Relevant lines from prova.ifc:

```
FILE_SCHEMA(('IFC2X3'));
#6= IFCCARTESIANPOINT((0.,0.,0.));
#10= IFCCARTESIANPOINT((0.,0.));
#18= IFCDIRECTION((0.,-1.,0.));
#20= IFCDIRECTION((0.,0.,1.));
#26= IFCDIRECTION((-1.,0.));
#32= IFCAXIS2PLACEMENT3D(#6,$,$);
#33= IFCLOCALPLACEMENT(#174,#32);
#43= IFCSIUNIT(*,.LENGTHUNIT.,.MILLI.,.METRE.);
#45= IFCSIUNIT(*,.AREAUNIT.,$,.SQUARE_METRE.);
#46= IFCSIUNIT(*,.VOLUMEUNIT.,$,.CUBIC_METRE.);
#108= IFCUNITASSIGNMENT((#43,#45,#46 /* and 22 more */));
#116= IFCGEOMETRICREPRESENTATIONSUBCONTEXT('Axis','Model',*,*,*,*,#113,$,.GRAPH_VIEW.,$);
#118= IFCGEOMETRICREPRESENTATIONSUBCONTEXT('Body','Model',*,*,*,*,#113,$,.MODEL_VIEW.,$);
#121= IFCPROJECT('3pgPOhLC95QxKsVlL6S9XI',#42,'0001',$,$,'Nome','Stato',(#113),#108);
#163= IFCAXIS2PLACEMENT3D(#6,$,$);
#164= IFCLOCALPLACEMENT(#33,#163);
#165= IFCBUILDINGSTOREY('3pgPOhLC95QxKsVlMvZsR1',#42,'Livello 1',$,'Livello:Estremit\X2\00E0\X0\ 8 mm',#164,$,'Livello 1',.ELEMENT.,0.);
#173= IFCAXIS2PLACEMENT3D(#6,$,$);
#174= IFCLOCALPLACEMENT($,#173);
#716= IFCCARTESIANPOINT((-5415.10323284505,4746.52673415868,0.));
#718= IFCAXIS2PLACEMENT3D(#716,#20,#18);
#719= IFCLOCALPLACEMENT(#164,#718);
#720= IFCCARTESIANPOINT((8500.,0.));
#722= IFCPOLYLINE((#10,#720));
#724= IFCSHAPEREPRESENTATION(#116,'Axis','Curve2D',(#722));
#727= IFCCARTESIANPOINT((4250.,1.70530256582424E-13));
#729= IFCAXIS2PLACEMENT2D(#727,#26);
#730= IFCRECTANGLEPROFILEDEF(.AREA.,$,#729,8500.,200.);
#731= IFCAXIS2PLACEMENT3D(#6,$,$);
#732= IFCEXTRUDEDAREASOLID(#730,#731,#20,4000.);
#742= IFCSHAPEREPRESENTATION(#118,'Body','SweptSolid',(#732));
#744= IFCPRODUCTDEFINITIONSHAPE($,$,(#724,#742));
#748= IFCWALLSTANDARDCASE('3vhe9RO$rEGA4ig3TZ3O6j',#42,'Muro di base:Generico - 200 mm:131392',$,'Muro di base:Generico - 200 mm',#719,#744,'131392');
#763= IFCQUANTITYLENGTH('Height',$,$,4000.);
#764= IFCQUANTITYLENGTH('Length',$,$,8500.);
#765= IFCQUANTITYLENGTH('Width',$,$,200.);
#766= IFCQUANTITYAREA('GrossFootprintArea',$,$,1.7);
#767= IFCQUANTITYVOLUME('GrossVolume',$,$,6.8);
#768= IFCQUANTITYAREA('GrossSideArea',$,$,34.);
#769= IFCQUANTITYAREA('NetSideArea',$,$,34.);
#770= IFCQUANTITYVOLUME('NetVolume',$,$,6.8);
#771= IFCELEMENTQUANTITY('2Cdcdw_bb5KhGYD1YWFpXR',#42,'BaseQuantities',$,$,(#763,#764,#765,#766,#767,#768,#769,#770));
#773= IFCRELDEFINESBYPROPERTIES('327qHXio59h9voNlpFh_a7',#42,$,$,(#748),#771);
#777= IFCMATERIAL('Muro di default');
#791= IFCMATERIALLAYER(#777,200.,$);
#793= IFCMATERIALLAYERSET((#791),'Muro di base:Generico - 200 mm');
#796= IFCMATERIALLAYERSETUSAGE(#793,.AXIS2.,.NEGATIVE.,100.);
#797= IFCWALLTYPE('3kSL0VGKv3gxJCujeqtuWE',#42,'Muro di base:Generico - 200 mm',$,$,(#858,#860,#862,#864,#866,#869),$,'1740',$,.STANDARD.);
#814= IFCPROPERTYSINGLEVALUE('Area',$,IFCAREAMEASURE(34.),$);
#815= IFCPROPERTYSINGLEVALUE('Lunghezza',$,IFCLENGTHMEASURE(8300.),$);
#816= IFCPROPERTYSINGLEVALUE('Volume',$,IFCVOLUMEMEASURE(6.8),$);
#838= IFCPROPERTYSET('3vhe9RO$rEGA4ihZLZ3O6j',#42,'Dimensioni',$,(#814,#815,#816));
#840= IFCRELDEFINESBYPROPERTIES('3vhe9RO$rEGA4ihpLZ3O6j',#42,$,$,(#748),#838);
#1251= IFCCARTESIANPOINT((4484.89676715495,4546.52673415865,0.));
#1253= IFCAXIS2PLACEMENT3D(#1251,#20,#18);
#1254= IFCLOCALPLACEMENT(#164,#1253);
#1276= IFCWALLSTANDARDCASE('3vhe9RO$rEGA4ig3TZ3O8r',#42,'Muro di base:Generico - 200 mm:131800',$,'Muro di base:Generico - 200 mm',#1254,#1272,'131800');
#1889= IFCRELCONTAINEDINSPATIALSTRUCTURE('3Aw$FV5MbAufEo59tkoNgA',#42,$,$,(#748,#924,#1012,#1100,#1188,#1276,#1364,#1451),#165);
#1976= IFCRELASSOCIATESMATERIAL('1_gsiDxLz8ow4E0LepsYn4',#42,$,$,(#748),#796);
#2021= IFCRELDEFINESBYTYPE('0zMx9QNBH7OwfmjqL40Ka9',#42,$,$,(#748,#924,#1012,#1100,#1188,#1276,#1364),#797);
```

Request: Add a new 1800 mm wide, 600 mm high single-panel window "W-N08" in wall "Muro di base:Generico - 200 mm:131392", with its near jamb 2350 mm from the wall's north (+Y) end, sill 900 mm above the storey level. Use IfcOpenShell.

```python
import numpy as np
import ifcopenshell
import ifcopenshell.api.feature
import ifcopenshell.api.geometry
import ifcopenshell.api.pset
import ifcopenshell.api.root
import ifcopenshell.api.spatial
import ifcopenshell.api.type
import ifcopenshell.geom
import ifcopenshell.util.element
import ifcopenshell.util.placement
import ifcopenshell.util.representation
import ifcopenshell.util.shape
import ifcopenshell.util.unit

model = ifcopenshell.open("prova.ifc")
unit_scale = ifcopenshell.util.unit.calculate_unit_scale(model)
area_scale = ifcopenshell.util.unit.calculate_unit_scale(model, "AREAUNIT")
volume_scale = ifcopenshell.util.unit.calculate_unit_scale(model, "VOLUMEUNIT")
settings = ifcopenshell.geom.settings()


def volume(element):
    """Net volume in cubic metres, openings subtracted."""
    shape = ifcopenshell.geom.create_shape(settings, element)
    return ifcopenshell.util.shape.get_volume(shape.geometry)


wall = model.by_guid("3vhe9RO$rEGA4ig3TZ3O6j")
storey = ifcopenshell.util.element.get_container(wall, ifc_class="IfcBuildingStorey")
context = ifcopenshell.util.representation.get_context(model, "Model", "Body", "MODEL_VIEW")
before = volume(wall)

width, height, from_end, sill = 1.8, 0.6, 2.35, 0.9  # metres

# The wall runs along its own X axis, and the end named is its -X end.
wall_shape = ifcopenshell.geom.create_shape(settings, wall)
x, y, z = ifcopenshell.util.shape.get_vertices(wall_shape.geometry).T
start = x.min() + from_end
face, thickness = float(y.min()), float(y.max() - y.min())
wall_matrix = ifcopenshell.util.placement.get_local_placement(wall.ObjectPlacement)
level = ifcopenshell.util.placement.get_local_placement(storey.ObjectPlacement)[2, 3]


def in_wall(x, y):
    """Placement at x, y metres in the wall's axes, at sill height."""
    matrix = wall_matrix.copy()
    matrix[:, 3] = wall_matrix @ np.array([x / unit_scale, y / unit_scale, 0.0, 1.0])
    matrix[2, 3] = level + sill / unit_scale
    return matrix


# Opening: a box that overshoots both wall faces by 50 mm.
opening = ifcopenshell.api.root.create_entity(model, ifc_class="IfcOpeningElement")
box = ifcopenshell.api.geometry.add_wall_representation(
    model, context=context, length=width, height=height, thickness=thickness + 0.1
)
ifcopenshell.api.geometry.assign_representation(model, product=opening, representation=box)
ifcopenshell.api.geometry.edit_object_placement(model, product=opening, matrix=in_wall(start, face - 0.05), is_si=False)
ifcopenshell.api.feature.add_feature(model, feature=opening, element=wall)

window = ifcopenshell.api.root.create_entity(model, ifc_class="IfcWindow", name="W-N08")
window.OverallWidth, window.OverallHeight = width / unit_scale, height / unit_scale
body = ifcopenshell.api.geometry.add_window_representation(
    model,
    context=context,
    overall_width=window.OverallWidth,
    overall_height=window.OverallHeight,
    partition_type="SINGLE_PANEL",
)
ifcopenshell.api.geometry.assign_representation(model, product=window, representation=body)
ifcopenshell.api.spatial.assign_container(model, products=[window], relating_structure=storey)
fills = ifcopenshell.api.feature.add_filling(model, opening=opening, element=window)
fills.OwnerHistory = window.OwnerHistory  # required in IFC2X3

# IFC2X3 keeps the operation on the window style.
style = ifcopenshell.api.root.create_entity(model, ifc_class="IfcWindowStyle", name="W-N08")
style.OperationType, style.ConstructionType = "SINGLE_PANEL", "NOTDEFINED"
style.ParameterTakesPrecedence = style.Sizeable = False
ifcopenshell.api.type.assign_type(model, related_objects=[window], relating_type=style)

# Centre the window in the wall's thickness.
ifcopenshell.api.geometry.edit_object_placement(model, product=window, matrix=in_wall(start, face), is_si=False)
window_shape = ifcopenshell.geom.create_shape(settings, window)
depth = ifcopenshell.util.shape.get_vertices(window_shape.geometry)[:, 1]
offset = face + thickness / 2 - (depth.min() + depth.max()) / 2
ifcopenshell.api.geometry.edit_object_placement(model, product=window, matrix=in_wall(start, offset), is_si=False)

after = volume(wall)

# Update the wall's stored quantities.
qto = model.by_id(ifcopenshell.util.element.get_pset(wall, "BaseQuantities", should_inherit=False)["id"])
ifcopenshell.api.pset.edit_qto(model, qto=qto, properties={
    "NetSideArea": after / thickness / area_scale,
    "NetVolume": after / volume_scale,
})
pset = model.by_id(ifcopenshell.util.element.get_pset(wall, "Dimensioni", should_inherit=False)["id"])
ifcopenshell.api.pset.edit_pset(model, pset=pset, properties={
    "Area": model.create_entity("IfcAreaMeasure", after / thickness / area_scale),
    "Volume": model.create_entity("IfcVolumeMeasure", after / volume_scale),
})

print(f"wall volume {before:.3f} -> {after:.3f} m3")

model.write("prova_rev.ifc")
```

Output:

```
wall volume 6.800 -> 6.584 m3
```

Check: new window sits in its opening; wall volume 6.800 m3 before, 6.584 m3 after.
